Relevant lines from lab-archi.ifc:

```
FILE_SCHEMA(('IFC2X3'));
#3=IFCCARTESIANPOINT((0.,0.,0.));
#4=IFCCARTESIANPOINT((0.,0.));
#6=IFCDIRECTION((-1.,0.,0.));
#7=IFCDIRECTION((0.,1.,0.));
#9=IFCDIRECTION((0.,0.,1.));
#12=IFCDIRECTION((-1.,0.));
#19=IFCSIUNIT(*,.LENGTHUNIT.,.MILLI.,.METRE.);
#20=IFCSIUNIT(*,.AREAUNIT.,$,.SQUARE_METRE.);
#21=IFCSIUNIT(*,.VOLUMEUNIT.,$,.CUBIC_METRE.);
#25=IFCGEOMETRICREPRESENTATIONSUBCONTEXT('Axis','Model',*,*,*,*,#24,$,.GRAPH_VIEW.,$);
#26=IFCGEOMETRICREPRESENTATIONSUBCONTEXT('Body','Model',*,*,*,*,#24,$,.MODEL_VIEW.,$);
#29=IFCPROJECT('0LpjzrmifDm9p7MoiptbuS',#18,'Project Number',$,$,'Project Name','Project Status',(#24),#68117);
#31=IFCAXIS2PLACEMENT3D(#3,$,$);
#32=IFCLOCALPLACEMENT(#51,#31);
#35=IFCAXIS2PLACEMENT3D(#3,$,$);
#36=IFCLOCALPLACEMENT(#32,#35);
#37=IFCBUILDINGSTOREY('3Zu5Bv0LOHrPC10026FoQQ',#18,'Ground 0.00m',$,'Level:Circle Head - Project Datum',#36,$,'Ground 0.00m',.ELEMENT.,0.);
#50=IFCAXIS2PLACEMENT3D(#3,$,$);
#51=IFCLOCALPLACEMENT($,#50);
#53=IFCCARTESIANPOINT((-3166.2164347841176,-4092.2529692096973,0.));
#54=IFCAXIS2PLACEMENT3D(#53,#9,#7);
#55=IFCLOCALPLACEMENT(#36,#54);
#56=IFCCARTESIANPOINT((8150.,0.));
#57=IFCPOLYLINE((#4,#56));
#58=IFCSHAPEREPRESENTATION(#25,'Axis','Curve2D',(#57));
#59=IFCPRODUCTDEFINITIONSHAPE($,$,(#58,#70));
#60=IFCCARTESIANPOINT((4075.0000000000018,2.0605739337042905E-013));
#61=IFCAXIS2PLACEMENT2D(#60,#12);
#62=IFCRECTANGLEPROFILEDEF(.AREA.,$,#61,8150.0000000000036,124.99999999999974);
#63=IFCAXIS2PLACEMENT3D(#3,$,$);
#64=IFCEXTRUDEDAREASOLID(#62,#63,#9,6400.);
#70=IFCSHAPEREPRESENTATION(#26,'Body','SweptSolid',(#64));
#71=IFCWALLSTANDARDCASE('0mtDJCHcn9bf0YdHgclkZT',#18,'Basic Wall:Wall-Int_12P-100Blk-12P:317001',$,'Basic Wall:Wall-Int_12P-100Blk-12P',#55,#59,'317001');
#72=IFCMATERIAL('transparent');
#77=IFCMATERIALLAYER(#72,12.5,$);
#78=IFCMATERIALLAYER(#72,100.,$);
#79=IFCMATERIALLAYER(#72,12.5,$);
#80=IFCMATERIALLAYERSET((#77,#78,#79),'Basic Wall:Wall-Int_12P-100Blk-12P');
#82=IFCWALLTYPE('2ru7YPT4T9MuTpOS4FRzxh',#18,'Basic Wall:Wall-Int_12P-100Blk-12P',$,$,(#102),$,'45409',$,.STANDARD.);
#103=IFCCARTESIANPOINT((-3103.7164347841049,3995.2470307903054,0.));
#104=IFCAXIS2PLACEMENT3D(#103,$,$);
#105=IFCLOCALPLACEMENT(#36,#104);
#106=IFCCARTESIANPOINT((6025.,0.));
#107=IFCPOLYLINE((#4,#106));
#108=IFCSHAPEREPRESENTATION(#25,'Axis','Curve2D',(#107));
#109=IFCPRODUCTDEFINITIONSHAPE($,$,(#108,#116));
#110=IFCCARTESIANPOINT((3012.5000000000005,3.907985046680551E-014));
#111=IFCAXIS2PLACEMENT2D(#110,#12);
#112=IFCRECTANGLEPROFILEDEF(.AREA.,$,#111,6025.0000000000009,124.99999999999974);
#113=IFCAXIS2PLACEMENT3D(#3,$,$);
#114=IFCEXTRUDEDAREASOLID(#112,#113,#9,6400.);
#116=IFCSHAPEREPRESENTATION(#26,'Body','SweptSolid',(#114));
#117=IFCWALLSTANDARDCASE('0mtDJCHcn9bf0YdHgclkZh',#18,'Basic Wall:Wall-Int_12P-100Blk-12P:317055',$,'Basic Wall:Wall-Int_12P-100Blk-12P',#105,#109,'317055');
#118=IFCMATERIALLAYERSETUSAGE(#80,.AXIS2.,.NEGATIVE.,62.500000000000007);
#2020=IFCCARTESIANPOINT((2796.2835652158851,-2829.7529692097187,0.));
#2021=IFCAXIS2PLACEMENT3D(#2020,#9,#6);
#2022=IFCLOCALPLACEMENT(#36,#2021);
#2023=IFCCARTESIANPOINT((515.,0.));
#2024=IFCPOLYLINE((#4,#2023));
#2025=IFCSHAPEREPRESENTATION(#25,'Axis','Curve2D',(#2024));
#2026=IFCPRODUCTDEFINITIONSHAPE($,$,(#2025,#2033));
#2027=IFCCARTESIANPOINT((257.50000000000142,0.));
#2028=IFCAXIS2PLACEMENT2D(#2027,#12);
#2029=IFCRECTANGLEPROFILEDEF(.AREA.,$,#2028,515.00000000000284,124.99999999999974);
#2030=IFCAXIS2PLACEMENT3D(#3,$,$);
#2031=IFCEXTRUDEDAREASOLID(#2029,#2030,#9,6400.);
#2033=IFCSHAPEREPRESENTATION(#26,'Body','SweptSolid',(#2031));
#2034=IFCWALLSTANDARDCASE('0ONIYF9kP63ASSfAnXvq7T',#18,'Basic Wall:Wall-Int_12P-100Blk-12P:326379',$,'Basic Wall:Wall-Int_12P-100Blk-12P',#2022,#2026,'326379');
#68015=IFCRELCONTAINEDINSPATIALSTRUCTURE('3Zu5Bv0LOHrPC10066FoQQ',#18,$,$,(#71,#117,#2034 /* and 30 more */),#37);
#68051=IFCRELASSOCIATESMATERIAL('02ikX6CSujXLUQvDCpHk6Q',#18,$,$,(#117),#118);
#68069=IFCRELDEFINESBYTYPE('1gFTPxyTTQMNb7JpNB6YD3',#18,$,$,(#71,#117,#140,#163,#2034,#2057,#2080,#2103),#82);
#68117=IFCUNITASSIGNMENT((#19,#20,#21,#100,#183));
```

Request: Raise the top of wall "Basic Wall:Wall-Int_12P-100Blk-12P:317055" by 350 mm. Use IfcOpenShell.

```python
import ifcopenshell
import ifcopenshell.geom
import ifcopenshell.util.representation
import ifcopenshell.util.shape
import ifcopenshell.util.unit

model = ifcopenshell.open("lab-archi.ifc")
unit_scale = ifcopenshell.util.unit.calculate_unit_scale(model)
settings = ifcopenshell.geom.settings()


def volume(element):
    """Net volume in cubic metres, openings subtracted."""
    shape = ifcopenshell.geom.create_shape(settings, element)
    return ifcopenshell.util.shape.get_volume(shape.geometry)


wall = model.by_id(117)
before = volume(wall)

body = ifcopenshell.util.representation.get_representation(wall, "Model", "Body")
solid = body.Items[0]
old_height = solid.Depth
solid.Depth += 0.35 / unit_scale
after = volume(wall)

print(f"height {old_height:g} -> {solid.Depth:g}, volume {before:.3f} -> {after:.3f} m3")

model.write("lab-archi_rev.ifc")
```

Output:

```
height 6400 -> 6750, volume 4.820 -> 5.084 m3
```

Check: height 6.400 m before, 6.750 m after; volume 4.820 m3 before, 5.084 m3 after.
